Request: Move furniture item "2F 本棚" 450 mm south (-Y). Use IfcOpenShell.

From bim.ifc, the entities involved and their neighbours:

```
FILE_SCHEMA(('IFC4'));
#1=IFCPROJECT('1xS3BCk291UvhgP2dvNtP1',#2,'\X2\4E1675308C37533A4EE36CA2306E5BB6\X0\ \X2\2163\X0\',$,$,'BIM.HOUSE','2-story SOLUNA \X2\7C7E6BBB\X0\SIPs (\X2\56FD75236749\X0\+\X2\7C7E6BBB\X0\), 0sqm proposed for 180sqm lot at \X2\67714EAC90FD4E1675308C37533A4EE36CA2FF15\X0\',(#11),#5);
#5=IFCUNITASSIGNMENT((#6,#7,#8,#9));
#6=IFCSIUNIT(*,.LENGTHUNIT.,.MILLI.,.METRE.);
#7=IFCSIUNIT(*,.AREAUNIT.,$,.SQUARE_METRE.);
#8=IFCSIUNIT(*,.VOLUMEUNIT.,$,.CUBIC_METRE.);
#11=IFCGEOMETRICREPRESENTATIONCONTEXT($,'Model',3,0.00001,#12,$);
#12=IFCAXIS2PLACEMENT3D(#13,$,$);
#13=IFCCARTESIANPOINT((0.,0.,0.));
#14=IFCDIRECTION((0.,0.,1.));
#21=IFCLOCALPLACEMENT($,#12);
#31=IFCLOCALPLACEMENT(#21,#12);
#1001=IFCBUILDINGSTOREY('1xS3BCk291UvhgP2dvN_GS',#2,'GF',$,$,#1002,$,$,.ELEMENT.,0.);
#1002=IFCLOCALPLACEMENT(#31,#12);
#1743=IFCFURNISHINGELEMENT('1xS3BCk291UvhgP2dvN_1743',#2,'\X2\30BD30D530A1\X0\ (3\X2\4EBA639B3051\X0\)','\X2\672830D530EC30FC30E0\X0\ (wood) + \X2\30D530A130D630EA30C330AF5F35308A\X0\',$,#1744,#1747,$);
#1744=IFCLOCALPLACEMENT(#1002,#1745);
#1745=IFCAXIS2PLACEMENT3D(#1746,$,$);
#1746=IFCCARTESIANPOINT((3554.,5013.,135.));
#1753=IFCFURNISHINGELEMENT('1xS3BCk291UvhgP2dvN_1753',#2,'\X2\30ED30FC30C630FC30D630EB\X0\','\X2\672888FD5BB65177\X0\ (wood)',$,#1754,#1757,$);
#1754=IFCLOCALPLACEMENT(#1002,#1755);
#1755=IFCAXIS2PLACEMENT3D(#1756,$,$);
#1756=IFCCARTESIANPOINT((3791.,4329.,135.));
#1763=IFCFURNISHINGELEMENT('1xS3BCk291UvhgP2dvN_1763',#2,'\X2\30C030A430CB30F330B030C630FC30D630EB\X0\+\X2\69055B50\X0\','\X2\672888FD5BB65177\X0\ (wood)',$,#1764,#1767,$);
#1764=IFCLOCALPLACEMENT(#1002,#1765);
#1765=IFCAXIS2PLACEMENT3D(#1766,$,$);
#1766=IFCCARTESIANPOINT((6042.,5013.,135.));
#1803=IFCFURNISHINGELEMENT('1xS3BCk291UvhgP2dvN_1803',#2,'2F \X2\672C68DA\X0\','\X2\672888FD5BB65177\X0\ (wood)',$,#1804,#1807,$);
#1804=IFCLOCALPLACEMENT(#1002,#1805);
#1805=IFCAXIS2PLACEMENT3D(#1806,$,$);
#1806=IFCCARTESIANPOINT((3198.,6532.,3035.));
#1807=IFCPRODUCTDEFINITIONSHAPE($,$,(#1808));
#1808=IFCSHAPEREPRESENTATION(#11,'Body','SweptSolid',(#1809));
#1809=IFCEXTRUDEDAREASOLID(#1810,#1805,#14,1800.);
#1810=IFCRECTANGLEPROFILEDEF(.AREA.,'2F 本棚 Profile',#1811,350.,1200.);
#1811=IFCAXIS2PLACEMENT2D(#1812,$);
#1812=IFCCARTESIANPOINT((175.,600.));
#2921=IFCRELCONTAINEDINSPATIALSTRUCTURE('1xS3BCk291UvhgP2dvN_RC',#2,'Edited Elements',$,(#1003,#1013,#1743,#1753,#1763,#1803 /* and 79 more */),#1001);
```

```python
import ifcopenshell
import ifcopenshell.api.geometry
import ifcopenshell.util.placement
import ifcopenshell.util.unit

model = ifcopenshell.open("bim.ifc")
unit_scale = ifcopenshell.util.unit.calculate_unit_scale(model)

item = model.by_guid("1xS3BCk291UvhgP2dvN_1803")
matrix = ifcopenshell.util.placement.get_local_placement(item.ObjectPlacement)
matrix[1, 3] -= 0.45 / unit_scale
ifcopenshell.api.geometry.edit_object_placement(model, product=item, matrix=matrix, is_si=False)

print(ifcopenshell.util.placement.get_local_placement(item.ObjectPlacement).round(3) + 0.0)

model.write("bim_rev.ifc")
```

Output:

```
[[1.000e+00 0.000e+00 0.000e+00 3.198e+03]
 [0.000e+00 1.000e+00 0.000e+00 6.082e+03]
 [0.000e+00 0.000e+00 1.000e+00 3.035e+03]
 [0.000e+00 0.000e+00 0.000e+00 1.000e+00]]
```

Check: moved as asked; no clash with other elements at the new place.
